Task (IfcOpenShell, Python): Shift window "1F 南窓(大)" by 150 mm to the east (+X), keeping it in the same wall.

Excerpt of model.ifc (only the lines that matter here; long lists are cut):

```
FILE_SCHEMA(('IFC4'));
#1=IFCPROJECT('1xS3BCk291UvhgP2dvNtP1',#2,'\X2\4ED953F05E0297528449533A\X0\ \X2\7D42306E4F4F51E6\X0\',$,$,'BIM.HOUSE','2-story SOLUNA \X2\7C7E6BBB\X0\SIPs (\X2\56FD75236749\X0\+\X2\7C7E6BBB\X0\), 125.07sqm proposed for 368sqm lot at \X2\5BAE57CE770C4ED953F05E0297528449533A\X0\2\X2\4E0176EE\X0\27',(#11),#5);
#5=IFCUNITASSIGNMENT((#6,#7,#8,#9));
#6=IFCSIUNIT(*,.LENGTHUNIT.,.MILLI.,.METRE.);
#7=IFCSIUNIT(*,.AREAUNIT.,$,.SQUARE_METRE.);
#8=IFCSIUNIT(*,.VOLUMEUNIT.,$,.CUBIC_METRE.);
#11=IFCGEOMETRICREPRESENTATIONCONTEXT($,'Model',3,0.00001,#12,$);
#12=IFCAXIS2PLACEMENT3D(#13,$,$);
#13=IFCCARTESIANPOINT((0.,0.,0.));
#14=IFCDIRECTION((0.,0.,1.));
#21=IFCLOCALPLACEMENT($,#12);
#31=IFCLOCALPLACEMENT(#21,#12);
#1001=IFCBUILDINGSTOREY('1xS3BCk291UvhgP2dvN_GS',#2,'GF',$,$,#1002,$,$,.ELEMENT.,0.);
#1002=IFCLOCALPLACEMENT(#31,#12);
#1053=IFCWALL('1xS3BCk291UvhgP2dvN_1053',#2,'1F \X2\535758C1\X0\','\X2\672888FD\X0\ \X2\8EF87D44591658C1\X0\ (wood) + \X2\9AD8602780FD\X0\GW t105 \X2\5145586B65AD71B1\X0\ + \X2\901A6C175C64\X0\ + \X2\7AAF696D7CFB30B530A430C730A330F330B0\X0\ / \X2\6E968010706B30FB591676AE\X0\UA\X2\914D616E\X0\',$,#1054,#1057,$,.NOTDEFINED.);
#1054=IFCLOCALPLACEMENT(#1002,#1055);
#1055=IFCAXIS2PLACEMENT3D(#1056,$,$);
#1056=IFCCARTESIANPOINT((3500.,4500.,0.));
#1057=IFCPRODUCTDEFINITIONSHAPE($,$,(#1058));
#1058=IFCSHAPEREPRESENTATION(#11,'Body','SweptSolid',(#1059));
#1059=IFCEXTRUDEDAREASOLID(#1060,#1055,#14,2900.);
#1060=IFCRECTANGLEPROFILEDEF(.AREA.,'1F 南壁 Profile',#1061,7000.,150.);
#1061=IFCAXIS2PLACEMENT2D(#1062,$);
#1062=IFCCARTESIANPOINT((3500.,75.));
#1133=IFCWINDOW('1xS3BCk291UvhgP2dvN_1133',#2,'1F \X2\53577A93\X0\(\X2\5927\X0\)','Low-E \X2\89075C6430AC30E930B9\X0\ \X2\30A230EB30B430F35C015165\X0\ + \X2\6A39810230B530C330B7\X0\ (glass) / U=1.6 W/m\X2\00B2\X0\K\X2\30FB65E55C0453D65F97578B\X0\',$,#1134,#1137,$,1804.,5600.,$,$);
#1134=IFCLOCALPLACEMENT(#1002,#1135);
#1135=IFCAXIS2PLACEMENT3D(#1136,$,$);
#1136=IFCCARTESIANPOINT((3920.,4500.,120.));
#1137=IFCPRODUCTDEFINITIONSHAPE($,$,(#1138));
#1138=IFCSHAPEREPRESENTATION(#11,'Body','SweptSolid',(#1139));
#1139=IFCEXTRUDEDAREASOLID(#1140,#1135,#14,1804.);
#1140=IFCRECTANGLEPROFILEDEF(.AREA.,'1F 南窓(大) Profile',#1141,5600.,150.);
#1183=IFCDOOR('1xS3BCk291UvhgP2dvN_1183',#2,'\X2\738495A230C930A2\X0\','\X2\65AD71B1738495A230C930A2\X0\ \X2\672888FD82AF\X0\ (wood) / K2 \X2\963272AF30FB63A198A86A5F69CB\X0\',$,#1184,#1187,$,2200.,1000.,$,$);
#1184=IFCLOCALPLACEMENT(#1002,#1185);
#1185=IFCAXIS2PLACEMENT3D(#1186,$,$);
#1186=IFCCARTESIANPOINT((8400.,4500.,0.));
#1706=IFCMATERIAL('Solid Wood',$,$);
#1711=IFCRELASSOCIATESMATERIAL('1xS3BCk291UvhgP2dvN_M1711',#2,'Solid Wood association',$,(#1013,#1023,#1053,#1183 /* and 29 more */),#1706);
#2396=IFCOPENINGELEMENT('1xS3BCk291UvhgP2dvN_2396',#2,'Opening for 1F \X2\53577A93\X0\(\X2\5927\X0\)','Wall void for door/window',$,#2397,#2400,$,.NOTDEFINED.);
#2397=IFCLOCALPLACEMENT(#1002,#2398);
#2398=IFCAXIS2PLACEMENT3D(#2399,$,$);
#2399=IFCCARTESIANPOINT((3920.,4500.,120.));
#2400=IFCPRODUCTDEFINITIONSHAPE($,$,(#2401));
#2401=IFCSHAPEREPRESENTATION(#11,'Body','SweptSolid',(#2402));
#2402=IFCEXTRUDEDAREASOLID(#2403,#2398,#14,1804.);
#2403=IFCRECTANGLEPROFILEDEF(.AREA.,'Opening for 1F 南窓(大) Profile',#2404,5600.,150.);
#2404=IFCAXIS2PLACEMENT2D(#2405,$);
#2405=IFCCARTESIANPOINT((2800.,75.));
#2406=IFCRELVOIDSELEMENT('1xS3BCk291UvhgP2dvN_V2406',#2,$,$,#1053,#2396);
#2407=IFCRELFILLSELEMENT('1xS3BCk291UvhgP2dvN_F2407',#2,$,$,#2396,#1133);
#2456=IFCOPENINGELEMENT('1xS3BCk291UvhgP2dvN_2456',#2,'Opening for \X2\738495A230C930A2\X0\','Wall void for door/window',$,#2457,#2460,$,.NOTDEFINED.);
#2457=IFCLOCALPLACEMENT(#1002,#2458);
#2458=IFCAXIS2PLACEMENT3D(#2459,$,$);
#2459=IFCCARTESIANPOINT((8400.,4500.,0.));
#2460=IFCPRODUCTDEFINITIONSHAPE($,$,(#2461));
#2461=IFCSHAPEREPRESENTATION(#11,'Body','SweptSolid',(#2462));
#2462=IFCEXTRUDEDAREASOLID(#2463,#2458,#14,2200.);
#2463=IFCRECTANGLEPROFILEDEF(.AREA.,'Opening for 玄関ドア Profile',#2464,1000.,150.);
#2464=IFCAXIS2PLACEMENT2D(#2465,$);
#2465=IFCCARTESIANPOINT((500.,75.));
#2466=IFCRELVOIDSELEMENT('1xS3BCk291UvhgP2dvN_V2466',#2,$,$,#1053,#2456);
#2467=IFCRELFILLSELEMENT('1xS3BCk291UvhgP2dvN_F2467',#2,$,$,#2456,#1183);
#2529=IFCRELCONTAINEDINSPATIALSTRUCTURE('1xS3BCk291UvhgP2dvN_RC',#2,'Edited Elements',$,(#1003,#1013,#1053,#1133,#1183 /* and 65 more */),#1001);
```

```python
import ifcopenshell
import ifcopenshell.api.geometry
import ifcopenshell.util.placement
import ifcopenshell.util.unit

model = ifcopenshell.open("model.ifc")
unit_scale = ifcopenshell.util.unit.calculate_unit_scale(model)

window = model.by_id(1133)
opening = window.FillsVoids[0].RelatingOpeningElement
wall = opening.VoidsElements[0].RelatingBuildingElement

wall_matrix = ifcopenshell.util.placement.get_local_placement(wall.ObjectPlacement)
shift = wall_matrix[:3, 0] * 0.15 / unit_scale
before = ifcopenshell.util.placement.get_local_placement(window.ObjectPlacement)[:3, 3].copy()

# The window is not placed relative to its opening, so move both.
for product in (opening, window):
    matrix = ifcopenshell.util.placement.get_local_placement(product.ObjectPlacement)
    matrix[:3, 3] += shift
    ifcopenshell.api.geometry.edit_object_placement(model, product=product, matrix=matrix, is_si=False)

after = ifcopenshell.util.placement.get_local_placement(window.ObjectPlacement)[:3, 3]
print("window moved by", (after - before).round(3) + 0.0)

model.write("model_updated.ifc")
```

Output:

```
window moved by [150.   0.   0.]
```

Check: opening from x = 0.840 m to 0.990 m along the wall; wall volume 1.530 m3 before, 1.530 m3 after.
